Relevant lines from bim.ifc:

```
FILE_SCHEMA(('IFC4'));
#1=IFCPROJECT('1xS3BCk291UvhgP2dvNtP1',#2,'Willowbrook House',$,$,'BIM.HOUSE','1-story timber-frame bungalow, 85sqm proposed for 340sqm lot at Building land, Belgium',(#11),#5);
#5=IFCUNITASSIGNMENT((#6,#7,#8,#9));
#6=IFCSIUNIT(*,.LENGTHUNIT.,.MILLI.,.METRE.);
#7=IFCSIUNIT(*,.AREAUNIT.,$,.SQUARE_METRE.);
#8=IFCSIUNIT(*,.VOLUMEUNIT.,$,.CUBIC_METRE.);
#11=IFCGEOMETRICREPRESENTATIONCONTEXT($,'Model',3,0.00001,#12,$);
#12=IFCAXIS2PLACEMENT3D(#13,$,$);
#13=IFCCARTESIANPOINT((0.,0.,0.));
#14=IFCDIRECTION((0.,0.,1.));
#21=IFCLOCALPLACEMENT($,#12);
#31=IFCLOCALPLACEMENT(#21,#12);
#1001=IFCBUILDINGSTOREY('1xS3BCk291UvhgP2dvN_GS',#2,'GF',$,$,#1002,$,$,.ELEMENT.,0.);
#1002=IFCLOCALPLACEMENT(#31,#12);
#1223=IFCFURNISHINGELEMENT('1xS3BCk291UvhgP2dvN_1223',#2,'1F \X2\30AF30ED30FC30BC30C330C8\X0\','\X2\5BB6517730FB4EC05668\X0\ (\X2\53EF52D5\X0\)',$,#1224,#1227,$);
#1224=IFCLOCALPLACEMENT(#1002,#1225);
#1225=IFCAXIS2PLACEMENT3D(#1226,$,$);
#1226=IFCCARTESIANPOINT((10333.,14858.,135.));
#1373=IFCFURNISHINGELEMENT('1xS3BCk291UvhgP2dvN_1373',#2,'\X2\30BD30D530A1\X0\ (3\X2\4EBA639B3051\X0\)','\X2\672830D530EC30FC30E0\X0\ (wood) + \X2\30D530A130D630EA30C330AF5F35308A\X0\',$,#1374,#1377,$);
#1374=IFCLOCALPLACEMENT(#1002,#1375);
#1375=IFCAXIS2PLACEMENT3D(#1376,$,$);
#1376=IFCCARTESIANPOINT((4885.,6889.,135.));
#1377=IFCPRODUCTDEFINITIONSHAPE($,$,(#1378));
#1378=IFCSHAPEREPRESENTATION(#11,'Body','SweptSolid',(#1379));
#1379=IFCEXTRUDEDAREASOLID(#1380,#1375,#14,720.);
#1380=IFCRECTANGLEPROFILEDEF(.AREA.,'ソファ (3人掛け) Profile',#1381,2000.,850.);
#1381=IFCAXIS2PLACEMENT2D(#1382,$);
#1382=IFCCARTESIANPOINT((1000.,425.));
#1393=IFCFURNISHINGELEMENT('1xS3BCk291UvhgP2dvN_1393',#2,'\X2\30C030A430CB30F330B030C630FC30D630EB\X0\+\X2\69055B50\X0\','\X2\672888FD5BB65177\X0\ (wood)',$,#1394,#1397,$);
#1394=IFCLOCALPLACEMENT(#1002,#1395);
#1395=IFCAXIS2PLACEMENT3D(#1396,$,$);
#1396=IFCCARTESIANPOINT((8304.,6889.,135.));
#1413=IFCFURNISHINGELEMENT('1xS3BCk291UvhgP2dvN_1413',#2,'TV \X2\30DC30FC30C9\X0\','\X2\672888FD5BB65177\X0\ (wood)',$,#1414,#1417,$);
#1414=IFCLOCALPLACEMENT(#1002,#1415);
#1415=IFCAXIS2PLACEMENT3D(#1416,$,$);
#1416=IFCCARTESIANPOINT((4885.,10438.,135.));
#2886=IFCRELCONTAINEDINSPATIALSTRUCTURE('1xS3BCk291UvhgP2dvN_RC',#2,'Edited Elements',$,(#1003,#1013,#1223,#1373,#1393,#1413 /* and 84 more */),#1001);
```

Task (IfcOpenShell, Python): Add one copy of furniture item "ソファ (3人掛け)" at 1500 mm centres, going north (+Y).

```python
import numpy as np
import ifcopenshell
import ifcopenshell.api.geometry
import ifcopenshell.api.root
import ifcopenshell.util.element
import ifcopenshell.util.placement

model = ifcopenshell.open("bim.ifc")


def reuse_history(source, copy):
    """copy_class also copies each property set's owner history, people and application; keep the originals."""
    for rel in copy.IsDefinedBy:
        if rel.is_a("IfcRelDefinesByProperties") and (history := rel.RelatingPropertyDefinition.OwnerHistory):
            rel.RelatingPropertyDefinition.OwnerHistory = source.OwnerHistory
            ifcopenshell.util.element.remove_deep2(model, history)


source = model.by_guid("1xS3BCk291UvhgP2dvN_1373")
base = ifcopenshell.util.placement.get_local_placement(source.ObjectPlacement)
step = np.array([0.0, 1.0, 0.0]) * 1500.0

for i in range(1, 2):
    copy = ifcopenshell.api.root.copy_class(model, product=source)
    copy.Representation = ifcopenshell.util.element.copy_deep(
        model, source.Representation, exclude=["IfcGeometricRepresentationContext", "IfcRepresentationMap"]
    )
    reuse_history(source, copy)
    matrix = base.copy()
    matrix[:3, 3] += i * step
    print("added at", matrix[:3, 3].round(3) + 0.0)
    ifcopenshell.api.geometry.edit_object_placement(model, product=copy, matrix=matrix, is_si=False)

model.write("bim_rev.ifc")
```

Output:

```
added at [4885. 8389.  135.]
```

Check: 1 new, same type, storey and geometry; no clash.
